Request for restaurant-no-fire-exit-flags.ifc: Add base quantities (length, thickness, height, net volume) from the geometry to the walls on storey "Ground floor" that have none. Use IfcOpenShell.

First a look at what the model holds.

```python
import ifcopenshell
import ifcopenshell.util.element
import ifcopenshell.util.unit

model = ifcopenshell.open("restaurant-no-fire-exit-flags.ifc")
print(model.schema)
for unit_type in ("LENGTHUNIT", "AREAUNIT", "VOLUMEUNIT"):
    print(unit_type, ifcopenshell.util.unit.calculate_unit_scale(model, unit_type))
storey = next(s for s in model.by_type("IfcBuildingStorey") if s.Name == "Ground floor")
walls = [e for e in ifcopenshell.util.element.get_decomposition(storey) if e.is_a("IfcWall")]
for e in sorted(walls, key=lambda e: e.id()):
    print(e.id(), e.is_a(), e.Name, list(ifcopenshell.util.element.get_psets(e, qtos_only=True)), sep=" | ")
```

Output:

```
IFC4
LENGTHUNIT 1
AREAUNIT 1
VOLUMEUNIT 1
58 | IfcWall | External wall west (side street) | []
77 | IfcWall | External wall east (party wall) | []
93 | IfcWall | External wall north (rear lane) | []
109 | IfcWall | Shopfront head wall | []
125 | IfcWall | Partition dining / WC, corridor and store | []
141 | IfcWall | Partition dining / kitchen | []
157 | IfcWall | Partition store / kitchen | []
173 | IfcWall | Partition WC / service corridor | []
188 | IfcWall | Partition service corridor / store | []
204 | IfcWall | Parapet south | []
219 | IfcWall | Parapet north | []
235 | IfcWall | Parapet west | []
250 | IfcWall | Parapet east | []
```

```python
import ifcopenshell
import ifcopenshell.api.pset
import ifcopenshell.geom
import ifcopenshell.util.element
import ifcopenshell.util.shape
import ifcopenshell.util.unit

model = ifcopenshell.open("restaurant-no-fire-exit-flags.ifc")
unit_scale = ifcopenshell.util.unit.calculate_unit_scale(model)
volume_scale = ifcopenshell.util.unit.calculate_unit_scale(model, "VOLUMEUNIT")
settings = ifcopenshell.geom.settings()

storey = next(s for s in model.by_type("IfcBuildingStorey") if s.Name == "Ground floor")
walls = [e for e in ifcopenshell.util.element.get_decomposition(storey) if e.is_a("IfcWall")]

for e in sorted(walls, key=lambda e: e.id()):
    if ifcopenshell.util.element.get_psets(e, qtos_only=True, should_inherit=False):
        continue
    # Geometry comes back in metres, in the element's own axes.
    shape = ifcopenshell.geom.create_shape(settings, e)
    values = {
        "Length": ifcopenshell.util.shape.get_x(shape.geometry) / unit_scale,
        "Width": ifcopenshell.util.shape.get_y(shape.geometry) / unit_scale,
        "Height": ifcopenshell.util.shape.get_z(shape.geometry) / unit_scale,
        "NetVolume": ifcopenshell.util.shape.get_volume(shape.geometry) / volume_scale,
    }
    qto = ifcopenshell.api.pset.add_qto(model, product=e, name="Qto_WallBaseQuantities")
    ifcopenshell.api.pset.edit_qto(model, qto=qto, properties=values)
    print(e.id(), {k: round(v, 3) for k, v in values.items()})

model.write("restaurant-no-fire-exit-flags_edited.ifc")
```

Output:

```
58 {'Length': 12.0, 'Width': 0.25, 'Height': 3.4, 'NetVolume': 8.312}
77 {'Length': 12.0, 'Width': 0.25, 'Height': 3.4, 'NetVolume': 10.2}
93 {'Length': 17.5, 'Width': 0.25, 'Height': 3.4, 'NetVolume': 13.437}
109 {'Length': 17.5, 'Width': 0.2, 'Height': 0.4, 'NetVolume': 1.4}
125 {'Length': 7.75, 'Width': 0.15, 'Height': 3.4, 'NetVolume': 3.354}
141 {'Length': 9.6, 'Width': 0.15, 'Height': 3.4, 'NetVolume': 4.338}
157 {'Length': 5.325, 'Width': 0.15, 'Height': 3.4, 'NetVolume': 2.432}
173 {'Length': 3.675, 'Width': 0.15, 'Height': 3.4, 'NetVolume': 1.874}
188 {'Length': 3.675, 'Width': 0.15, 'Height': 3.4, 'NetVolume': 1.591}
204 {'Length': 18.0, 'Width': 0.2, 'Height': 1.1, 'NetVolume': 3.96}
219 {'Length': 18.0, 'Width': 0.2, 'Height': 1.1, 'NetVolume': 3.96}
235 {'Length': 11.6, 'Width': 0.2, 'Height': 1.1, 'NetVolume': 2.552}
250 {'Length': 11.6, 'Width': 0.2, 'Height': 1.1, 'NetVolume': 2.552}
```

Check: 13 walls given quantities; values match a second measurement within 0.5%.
